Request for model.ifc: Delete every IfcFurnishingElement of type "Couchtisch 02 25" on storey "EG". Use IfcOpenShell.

First a look at what the model holds.

```python
import ifcopenshell
import ifcopenshell.util.element

model = ifcopenshell.open("model.ifc")
print(model.schema)
storey = next(s for s in model.by_type("IfcBuildingStorey") if s.Name == "EG")
furniture = [e for e in ifcopenshell.util.element.get_decomposition(storey) if e.is_a("IfcFurnishingElement")]
seen = {}
for e in furniture:
    element_type = ifcopenshell.util.element.get_type(e)
    name = element_type.Name if element_type not in (None, e) else None
    seen[name] = seen.get(name, 0) + 1
for name, count in sorted(seen.items(), key=str):
    print(count, "x", name)
```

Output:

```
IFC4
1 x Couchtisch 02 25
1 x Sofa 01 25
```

```python
import ifcopenshell
import ifcopenshell.api.root
import ifcopenshell.util.element

model = ifcopenshell.open("model.ifc")

storey = next(s for s in model.by_type("IfcBuildingStorey") if s.Name == "EG")
furniture = [e for e in ifcopenshell.util.element.get_decomposition(storey) if e.is_a("IfcFurnishingElement")]
targets = [e for e in furniture if (t := ifcopenshell.util.element.get_type(e)) not in (None, e) and t.Name == "Couchtisch 02 25"]

for e in targets:
    ifcopenshell.api.root.remove_product(model, product=e)
print(len(targets), "removed")

model.write("model_updated.ifc")
```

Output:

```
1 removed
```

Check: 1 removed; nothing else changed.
